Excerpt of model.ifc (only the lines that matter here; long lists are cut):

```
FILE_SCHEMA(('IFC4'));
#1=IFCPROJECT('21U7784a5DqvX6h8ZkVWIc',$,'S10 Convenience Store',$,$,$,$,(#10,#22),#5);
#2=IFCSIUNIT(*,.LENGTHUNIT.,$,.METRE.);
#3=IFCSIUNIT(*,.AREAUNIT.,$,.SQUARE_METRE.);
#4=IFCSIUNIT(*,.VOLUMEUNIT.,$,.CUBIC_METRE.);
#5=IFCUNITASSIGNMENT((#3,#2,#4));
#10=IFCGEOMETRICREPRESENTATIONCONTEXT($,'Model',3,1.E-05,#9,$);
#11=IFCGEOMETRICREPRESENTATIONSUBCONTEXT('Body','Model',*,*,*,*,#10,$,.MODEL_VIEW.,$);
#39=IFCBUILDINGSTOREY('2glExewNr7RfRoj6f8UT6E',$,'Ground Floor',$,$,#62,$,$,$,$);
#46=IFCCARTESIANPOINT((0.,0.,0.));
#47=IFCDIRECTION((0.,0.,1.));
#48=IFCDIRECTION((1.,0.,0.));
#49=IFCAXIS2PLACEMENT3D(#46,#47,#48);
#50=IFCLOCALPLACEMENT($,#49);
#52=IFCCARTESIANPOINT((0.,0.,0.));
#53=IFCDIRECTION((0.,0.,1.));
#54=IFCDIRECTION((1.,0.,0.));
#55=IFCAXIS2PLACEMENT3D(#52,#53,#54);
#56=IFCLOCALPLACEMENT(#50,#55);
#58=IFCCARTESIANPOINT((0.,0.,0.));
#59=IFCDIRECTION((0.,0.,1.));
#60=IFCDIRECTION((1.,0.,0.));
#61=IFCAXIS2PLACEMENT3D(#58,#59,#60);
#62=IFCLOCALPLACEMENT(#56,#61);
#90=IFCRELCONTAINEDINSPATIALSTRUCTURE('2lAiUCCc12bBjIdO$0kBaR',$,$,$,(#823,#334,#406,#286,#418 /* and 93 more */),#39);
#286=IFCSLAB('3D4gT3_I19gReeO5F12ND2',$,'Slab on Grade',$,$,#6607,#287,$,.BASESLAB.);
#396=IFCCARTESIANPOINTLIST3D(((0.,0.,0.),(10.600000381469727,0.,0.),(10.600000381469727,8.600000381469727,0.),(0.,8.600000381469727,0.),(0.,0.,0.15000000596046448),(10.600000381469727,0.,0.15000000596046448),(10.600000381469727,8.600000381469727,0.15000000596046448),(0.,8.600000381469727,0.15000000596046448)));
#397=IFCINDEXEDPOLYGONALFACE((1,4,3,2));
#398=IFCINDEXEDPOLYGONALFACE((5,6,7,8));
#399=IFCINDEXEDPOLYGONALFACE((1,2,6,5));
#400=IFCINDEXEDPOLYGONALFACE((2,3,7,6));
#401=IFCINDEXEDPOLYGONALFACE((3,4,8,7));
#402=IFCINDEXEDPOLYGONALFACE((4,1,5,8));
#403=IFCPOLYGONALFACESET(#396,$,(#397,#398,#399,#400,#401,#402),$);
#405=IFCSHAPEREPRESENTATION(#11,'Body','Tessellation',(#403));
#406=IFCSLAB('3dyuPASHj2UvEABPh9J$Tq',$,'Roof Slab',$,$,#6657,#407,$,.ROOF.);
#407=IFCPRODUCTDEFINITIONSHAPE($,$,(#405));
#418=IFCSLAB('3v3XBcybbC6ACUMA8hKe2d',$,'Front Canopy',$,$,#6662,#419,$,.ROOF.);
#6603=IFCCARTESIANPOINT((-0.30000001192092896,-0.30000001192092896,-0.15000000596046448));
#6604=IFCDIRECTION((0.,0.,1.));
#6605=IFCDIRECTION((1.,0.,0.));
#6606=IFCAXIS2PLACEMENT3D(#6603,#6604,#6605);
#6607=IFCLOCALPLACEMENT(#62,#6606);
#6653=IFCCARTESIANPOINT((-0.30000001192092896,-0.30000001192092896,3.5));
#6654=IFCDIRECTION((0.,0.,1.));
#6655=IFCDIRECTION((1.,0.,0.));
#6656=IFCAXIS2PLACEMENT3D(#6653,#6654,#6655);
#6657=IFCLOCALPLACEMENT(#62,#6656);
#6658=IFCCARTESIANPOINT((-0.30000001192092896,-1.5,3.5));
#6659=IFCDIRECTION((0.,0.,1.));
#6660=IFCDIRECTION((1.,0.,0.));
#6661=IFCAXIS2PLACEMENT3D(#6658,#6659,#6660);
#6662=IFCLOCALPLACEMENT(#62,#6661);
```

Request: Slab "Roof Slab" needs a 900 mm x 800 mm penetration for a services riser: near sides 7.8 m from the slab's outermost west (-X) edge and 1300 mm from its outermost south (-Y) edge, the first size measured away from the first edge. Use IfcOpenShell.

```python
import numpy as np
import ifcopenshell
import ifcopenshell.api.feature
import ifcopenshell.api.geometry
import ifcopenshell.api.root
import ifcopenshell.geom
import ifcopenshell.util.placement
import ifcopenshell.util.representation
import ifcopenshell.util.shape
import ifcopenshell.util.unit

model = ifcopenshell.open("model.ifc")
unit_scale = ifcopenshell.util.unit.calculate_unit_scale(model)
settings = ifcopenshell.geom.settings()


def volume(element):
    """Net volume in cubic metres, openings subtracted."""
    shape = ifcopenshell.geom.create_shape(settings, element)
    return ifcopenshell.util.shape.get_volume(shape.geometry)


slab = model.by_guid("3dyuPASHj2UvEABPh9J$Tq")
before = volume(slab)

# Extent in the slab's own axes, in metres. The edges named are its -X and -Y sides.
slab_shape = ifcopenshell.geom.create_shape(settings, slab)
vertices = ifcopenshell.util.shape.get_vertices(slab_shape.geometry)
x_min, y_min, bottom = vertices.min(axis=0)
top = vertices[:, 2].max()

opening = ifcopenshell.api.root.create_entity(model, ifc_class="IfcOpeningElement", name="Services riser opening", predefined_type="OPENING")
context = ifcopenshell.util.representation.get_context(model, "Model", "Body", "MODEL_VIEW")
width, depth = 0.9, 0.8
outline = [(0.0, 0.0), (width, 0.0), (width, depth), (0.0, depth), (0.0, 0.0)]
# Overshoot both faces by 50 mm so the cut is clean.
shape = ifcopenshell.api.geometry.add_slab_representation(
    model, context=context, depth=top - bottom + 0.1, polyline=outline
)
ifcopenshell.api.geometry.assign_representation(model, product=opening, representation=shape)

matrix = ifcopenshell.util.placement.get_local_placement(slab.ObjectPlacement)
matrix[:, 3] = matrix @ np.append(np.array([x_min + 7.8, y_min + 1.3, bottom - 0.05]) / unit_scale, 1.0)
ifcopenshell.api.geometry.edit_object_placement(model, product=opening, matrix=matrix, is_si=False)
ifcopenshell.api.feature.add_feature(model, feature=opening, element=slab)

after = volume(slab)

print(f"slab volume {before:.3f} -> {after:.3f} m3")

model.write("model_updated.ifc")
```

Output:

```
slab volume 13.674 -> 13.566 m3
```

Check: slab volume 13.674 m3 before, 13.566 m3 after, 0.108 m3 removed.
